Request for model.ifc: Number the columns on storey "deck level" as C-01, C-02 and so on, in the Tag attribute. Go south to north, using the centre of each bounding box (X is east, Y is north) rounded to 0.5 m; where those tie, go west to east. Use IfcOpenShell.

First a look at what the model holds.

```python
import ifcopenshell
import ifcopenshell.util.element
import ifcopenshell.util.placement

model = ifcopenshell.open("model.ifc")
print(model.schema)
storey = next(s for s in model.by_type("IfcBuildingStorey") if s.Name == "deck level")
columns = [e for e in ifcopenshell.util.element.get_decomposition(storey) if e.is_a("IfcColumn")]
for e in sorted(columns, key=lambda e: e.id()):
    origin = ifcopenshell.util.placement.get_local_placement(e.ObjectPlacement)[:3, 3]
    print(e.id(), e.Tag, e.Name, origin.round(2) + 0.0, sep=" | ")
```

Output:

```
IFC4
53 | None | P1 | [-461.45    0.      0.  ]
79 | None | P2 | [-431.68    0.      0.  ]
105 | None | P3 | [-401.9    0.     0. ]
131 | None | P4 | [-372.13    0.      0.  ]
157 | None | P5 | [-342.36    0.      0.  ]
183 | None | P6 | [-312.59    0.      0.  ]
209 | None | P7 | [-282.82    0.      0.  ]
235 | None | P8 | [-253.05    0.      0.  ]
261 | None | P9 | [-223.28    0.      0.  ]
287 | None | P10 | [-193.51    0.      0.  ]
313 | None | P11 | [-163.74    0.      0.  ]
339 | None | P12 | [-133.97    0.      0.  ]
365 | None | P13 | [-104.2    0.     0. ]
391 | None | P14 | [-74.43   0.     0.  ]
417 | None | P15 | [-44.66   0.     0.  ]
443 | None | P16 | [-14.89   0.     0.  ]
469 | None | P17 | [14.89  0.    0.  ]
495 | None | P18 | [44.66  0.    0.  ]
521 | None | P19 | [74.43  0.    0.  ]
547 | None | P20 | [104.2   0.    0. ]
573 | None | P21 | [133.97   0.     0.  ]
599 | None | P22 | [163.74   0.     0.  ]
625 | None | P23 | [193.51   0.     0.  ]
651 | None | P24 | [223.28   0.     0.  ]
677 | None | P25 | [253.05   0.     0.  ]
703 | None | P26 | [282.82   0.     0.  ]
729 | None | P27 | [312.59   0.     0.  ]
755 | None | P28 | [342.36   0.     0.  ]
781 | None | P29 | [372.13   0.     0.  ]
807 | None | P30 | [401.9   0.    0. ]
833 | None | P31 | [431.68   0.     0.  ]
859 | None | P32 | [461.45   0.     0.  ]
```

```python
import ifcopenshell
import ifcopenshell.geom
import ifcopenshell.util.element
import ifcopenshell.util.shape

model = ifcopenshell.open("model.ifc")
settings = ifcopenshell.geom.settings()
settings.set("use-world-coords", True)


def centre(element):
    shape = ifcopenshell.geom.create_shape(settings, element)
    return ifcopenshell.util.shape.get_bbox_centroid(shape.geometry)


storey = next(s for s in model.by_type("IfcBuildingStorey") if s.Name == "deck level")
columns = [e for e in ifcopenshell.util.element.get_decomposition(storey) if e.is_a("IfcColumn")]

# Insertion points can sit at a corner or the storey origin, so sort by the geometry (in metres).
centres = {e: centre(e) for e in columns}
columns.sort(key=lambda e: (round(centres[e][1] / 0.5), centres[e][0]))

for i, e in enumerate(columns, start=1):
    number = f"C-{i:02d}"
    e.Tag = number
    print(e.id(), number)

model.write("model_rev.ifc")
```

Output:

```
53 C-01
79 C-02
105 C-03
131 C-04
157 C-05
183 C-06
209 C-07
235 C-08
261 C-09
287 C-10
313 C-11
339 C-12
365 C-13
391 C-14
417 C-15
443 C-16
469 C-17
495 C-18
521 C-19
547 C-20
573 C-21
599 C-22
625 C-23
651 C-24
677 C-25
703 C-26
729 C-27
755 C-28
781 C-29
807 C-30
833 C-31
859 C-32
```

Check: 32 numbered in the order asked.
